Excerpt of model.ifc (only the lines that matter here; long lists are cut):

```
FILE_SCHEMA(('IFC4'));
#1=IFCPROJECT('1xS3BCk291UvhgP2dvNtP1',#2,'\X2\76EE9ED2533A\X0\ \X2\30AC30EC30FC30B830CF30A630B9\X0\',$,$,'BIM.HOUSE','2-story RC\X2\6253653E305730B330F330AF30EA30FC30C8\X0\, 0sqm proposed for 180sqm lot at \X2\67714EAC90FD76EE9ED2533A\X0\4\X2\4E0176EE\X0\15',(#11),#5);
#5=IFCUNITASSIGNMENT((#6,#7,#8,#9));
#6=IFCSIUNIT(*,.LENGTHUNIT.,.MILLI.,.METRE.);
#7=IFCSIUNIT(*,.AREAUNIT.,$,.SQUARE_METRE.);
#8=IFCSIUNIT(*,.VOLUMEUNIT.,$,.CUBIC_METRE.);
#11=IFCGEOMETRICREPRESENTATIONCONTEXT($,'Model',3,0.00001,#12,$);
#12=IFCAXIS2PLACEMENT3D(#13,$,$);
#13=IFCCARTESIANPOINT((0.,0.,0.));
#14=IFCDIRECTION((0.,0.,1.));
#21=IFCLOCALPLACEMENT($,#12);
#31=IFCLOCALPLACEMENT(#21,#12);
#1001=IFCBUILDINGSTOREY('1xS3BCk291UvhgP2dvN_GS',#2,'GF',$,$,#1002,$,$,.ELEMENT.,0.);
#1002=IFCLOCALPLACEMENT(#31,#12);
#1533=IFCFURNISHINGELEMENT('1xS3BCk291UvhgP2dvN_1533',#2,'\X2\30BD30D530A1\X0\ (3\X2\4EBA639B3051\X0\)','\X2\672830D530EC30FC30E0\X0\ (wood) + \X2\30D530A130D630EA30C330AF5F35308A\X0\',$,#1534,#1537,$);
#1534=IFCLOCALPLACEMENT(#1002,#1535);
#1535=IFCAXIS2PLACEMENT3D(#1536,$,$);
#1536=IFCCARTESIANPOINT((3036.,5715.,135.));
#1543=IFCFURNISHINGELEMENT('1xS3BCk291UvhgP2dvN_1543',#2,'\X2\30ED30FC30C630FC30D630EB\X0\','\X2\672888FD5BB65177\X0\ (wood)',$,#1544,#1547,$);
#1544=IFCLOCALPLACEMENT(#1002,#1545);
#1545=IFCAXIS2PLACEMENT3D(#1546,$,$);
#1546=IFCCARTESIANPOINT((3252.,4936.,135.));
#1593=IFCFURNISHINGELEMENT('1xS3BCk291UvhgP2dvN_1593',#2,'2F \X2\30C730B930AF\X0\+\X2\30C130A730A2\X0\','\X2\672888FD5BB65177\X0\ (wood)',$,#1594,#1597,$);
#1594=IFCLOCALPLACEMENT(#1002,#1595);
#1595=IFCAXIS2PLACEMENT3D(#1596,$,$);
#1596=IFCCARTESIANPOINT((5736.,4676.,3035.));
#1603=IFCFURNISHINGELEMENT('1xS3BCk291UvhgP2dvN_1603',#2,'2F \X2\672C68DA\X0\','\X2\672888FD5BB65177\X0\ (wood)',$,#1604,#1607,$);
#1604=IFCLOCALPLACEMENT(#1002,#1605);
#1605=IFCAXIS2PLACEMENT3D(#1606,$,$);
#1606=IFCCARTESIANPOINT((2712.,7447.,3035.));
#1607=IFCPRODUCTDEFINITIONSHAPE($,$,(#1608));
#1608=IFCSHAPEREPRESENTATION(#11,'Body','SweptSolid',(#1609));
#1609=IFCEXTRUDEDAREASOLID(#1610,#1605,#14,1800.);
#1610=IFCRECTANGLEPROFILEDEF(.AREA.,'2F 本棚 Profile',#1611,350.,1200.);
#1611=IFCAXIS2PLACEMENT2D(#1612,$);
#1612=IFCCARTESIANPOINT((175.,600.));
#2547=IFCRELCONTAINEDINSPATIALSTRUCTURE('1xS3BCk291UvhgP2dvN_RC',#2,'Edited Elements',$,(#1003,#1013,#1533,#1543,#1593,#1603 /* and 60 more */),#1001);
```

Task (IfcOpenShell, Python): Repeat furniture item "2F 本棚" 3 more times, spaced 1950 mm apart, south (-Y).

```python
import numpy as np
import ifcopenshell
import ifcopenshell.api.geometry
import ifcopenshell.api.root
import ifcopenshell.util.element
import ifcopenshell.util.placement
import ifcopenshell.util.unit

model = ifcopenshell.open("model.ifc")
unit_scale = ifcopenshell.util.unit.calculate_unit_scale(model)


def reuse_history(source, copy):
    """copy_class also copies each property set's owner history, people and application; keep the originals."""
    for rel in copy.IsDefinedBy:
        if rel.is_a("IfcRelDefinesByProperties") and (history := rel.RelatingPropertyDefinition.OwnerHistory):
            rel.RelatingPropertyDefinition.OwnerHistory = source.OwnerHistory
            ifcopenshell.util.element.remove_deep2(model, history)


source = model.by_id(1603)
base = ifcopenshell.util.placement.get_local_placement(source.ObjectPlacement)
step = np.array([0.0, -1.0, 0.0]) * 1.95 / unit_scale

for i in range(1, 4):
    copy = ifcopenshell.api.root.copy_class(model, product=source)
    copy.Representation = ifcopenshell.util.element.copy_deep(
        model, source.Representation, exclude=["IfcGeometricRepresentationContext", "IfcRepresentationMap"]
    )
    reuse_history(source, copy)
    matrix = base.copy()
    matrix[:3, 3] += i * step
    print("added at", matrix[:3, 3].round(3) + 0.0)
    ifcopenshell.api.geometry.edit_object_placement(model, product=copy, matrix=matrix, is_si=False)

model.write("model_updated.ifc")
```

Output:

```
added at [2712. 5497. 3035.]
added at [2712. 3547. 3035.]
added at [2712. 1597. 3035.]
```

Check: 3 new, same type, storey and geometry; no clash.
